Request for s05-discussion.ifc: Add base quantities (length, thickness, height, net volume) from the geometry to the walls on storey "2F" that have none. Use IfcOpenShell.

First a look at what the model holds.

```python
import ifcopenshell
import ifcopenshell.util.element
import ifcopenshell.util.unit

model = ifcopenshell.open("s05-discussion.ifc")
print(model.schema)
for unit_type in ("LENGTHUNIT", "AREAUNIT", "VOLUMEUNIT"):
    print(unit_type, ifcopenshell.util.unit.calculate_unit_scale(model, unit_type))
storey = next(s for s in model.by_type("IfcBuildingStorey") if s.Name == "2F")
walls = [e for e in ifcopenshell.util.element.get_decomposition(storey) if e.is_a("IfcWall")]
for e in sorted(walls, key=lambda e: e.id()):
    print(e.id(), e.is_a(), e.Name, list(ifcopenshell.util.element.get_psets(e, qtos_only=True)), sep=" | ")
```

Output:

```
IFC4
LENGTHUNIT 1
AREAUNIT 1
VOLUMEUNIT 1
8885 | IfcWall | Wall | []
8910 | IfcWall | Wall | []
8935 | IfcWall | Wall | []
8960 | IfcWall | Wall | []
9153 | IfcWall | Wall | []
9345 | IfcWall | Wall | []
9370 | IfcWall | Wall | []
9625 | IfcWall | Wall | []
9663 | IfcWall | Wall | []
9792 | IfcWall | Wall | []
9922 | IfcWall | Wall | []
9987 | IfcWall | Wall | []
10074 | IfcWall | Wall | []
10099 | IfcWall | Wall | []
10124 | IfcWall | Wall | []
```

```python
import ifcopenshell
import ifcopenshell.api.pset
import ifcopenshell.geom
import ifcopenshell.util.element
import ifcopenshell.util.shape
import ifcopenshell.util.unit

model = ifcopenshell.open("s05-discussion.ifc")
unit_scale = ifcopenshell.util.unit.calculate_unit_scale(model)
volume_scale = ifcopenshell.util.unit.calculate_unit_scale(model, "VOLUMEUNIT")
settings = ifcopenshell.geom.settings()

storey = next(s for s in model.by_type("IfcBuildingStorey") if s.Name == "2F")
walls = [e for e in ifcopenshell.util.element.get_decomposition(storey) if e.is_a("IfcWall")]

for e in sorted(walls, key=lambda e: e.id()):
    if ifcopenshell.util.element.get_psets(e, qtos_only=True, should_inherit=False):
        continue
    # Geometry comes back in metres, in the element's own axes.
    shape = ifcopenshell.geom.create_shape(settings, e)
    values = {
        "Length": ifcopenshell.util.shape.get_x(shape.geometry) / unit_scale,
        "Width": ifcopenshell.util.shape.get_y(shape.geometry) / unit_scale,
        "Height": ifcopenshell.util.shape.get_z(shape.geometry) / unit_scale,
        "NetVolume": ifcopenshell.util.shape.get_volume(shape.geometry) / volume_scale,
    }
    qto = ifcopenshell.api.pset.add_qto(model, product=e, name="Qto_WallBaseQuantities")
    ifcopenshell.api.pset.edit_qto(model, qto=qto, properties=values)
    print(e.id(), {k: round(v, 3) for k, v in values.items()})

model.write("s05-discussion-out.ifc")
```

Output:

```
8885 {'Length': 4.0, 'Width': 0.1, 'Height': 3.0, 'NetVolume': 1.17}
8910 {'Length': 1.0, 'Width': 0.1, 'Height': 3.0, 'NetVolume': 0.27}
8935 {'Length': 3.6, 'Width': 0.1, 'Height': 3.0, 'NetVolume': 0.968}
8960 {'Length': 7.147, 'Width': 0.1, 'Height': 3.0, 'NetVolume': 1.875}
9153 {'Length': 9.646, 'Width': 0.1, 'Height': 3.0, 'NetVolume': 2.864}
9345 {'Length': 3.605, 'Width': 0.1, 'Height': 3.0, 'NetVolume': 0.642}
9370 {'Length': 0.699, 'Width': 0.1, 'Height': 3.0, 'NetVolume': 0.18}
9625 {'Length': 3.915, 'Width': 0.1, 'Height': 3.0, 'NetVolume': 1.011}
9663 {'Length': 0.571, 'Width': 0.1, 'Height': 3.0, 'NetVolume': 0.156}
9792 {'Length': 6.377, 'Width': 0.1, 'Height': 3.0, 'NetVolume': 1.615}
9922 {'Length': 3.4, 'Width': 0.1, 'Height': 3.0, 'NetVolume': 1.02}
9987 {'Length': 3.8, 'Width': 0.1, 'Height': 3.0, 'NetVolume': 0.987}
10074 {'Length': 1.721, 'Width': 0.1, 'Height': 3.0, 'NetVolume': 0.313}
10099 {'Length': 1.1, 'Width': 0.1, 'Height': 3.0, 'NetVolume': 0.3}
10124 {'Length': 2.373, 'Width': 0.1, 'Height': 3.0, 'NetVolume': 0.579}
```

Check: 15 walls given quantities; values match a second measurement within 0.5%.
